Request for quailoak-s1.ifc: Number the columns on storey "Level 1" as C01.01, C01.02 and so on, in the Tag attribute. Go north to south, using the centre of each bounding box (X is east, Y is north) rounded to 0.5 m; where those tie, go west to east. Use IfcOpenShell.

First a look at what the model holds.

```python
import ifcopenshell
import ifcopenshell.util.element
import ifcopenshell.util.placement

model = ifcopenshell.open("quailoak-s1.ifc")
print(model.schema)
storey = next(s for s in model.by_type("IfcBuildingStorey") if s.Name == "Level 1")
columns = [e for e in ifcopenshell.util.element.get_decomposition(storey) if e.is_a("IfcColumn")]
for e in sorted(columns, key=lambda e: e.id()):
    origin = ifcopenshell.util.placement.get_local_placement(e.ObjectPlacement)[:3, 3]
    print(e.id(), e.Tag, e.Name, origin.round(2) + 0.0, sep=" | ")
```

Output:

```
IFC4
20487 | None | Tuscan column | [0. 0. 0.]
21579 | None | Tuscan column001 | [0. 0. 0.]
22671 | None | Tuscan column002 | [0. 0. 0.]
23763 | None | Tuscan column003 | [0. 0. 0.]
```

```python
import ifcopenshell
import ifcopenshell.geom
import ifcopenshell.util.element
import ifcopenshell.util.shape

model = ifcopenshell.open("quailoak-s1.ifc")
settings = ifcopenshell.geom.settings()
settings.set("use-world-coords", True)


def centre(element):
    shape = ifcopenshell.geom.create_shape(settings, element)
    return ifcopenshell.util.shape.get_bbox_centroid(shape.geometry)


storey = next(s for s in model.by_type("IfcBuildingStorey") if s.Name == "Level 1")
columns = [e for e in ifcopenshell.util.element.get_decomposition(storey) if e.is_a("IfcColumn")]

# Insertion points can sit at a corner or the storey origin, so sort by the geometry (in metres).
centres = {e: centre(e) for e in columns}
columns.sort(key=lambda e: (-round(centres[e][1] / 0.5), centres[e][0]))

for i, e in enumerate(columns, start=1):
    number = f"C01.{i:02d}"
    e.Tag = number
    print(e.id(), number)

model.write("quailoak-s1_rev.ifc")
```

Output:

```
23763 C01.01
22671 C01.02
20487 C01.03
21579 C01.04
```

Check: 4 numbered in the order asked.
